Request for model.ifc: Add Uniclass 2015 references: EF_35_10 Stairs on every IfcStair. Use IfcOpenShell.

First a look at what the model holds.

```python
import ifcopenshell

model = ifcopenshell.open("model.ifc")
print(model.schema)
print("classifications:", [c.Name for c in model.by_type("IfcClassification")])
for ifc_class in ("IfcDoor", "IfcRoof", "IfcStair", "IfcWall", "IfcWindow"):
    print(ifc_class, len(model.by_type(ifc_class)))
```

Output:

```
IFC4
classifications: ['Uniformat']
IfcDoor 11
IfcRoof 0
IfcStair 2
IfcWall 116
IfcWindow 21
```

```python
import ifcopenshell
import ifcopenshell.api.classification

model = ifcopenshell.open("model.ifc")

system = ifcopenshell.api.classification.add_classification(model, classification="Uniclass 2015")

codes = {
    "IfcStair": ("EF_35_10", "Stairs"),
}
for ifc_class, (code, name) in codes.items():
    products = model.by_type(ifc_class)
    ifcopenshell.api.classification.add_reference(
        model, products=products, classification=system, identification=code, name=name
    )
    print(code, len(products))

model.write("model_rev.ifc")
```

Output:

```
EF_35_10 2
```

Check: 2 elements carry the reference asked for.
